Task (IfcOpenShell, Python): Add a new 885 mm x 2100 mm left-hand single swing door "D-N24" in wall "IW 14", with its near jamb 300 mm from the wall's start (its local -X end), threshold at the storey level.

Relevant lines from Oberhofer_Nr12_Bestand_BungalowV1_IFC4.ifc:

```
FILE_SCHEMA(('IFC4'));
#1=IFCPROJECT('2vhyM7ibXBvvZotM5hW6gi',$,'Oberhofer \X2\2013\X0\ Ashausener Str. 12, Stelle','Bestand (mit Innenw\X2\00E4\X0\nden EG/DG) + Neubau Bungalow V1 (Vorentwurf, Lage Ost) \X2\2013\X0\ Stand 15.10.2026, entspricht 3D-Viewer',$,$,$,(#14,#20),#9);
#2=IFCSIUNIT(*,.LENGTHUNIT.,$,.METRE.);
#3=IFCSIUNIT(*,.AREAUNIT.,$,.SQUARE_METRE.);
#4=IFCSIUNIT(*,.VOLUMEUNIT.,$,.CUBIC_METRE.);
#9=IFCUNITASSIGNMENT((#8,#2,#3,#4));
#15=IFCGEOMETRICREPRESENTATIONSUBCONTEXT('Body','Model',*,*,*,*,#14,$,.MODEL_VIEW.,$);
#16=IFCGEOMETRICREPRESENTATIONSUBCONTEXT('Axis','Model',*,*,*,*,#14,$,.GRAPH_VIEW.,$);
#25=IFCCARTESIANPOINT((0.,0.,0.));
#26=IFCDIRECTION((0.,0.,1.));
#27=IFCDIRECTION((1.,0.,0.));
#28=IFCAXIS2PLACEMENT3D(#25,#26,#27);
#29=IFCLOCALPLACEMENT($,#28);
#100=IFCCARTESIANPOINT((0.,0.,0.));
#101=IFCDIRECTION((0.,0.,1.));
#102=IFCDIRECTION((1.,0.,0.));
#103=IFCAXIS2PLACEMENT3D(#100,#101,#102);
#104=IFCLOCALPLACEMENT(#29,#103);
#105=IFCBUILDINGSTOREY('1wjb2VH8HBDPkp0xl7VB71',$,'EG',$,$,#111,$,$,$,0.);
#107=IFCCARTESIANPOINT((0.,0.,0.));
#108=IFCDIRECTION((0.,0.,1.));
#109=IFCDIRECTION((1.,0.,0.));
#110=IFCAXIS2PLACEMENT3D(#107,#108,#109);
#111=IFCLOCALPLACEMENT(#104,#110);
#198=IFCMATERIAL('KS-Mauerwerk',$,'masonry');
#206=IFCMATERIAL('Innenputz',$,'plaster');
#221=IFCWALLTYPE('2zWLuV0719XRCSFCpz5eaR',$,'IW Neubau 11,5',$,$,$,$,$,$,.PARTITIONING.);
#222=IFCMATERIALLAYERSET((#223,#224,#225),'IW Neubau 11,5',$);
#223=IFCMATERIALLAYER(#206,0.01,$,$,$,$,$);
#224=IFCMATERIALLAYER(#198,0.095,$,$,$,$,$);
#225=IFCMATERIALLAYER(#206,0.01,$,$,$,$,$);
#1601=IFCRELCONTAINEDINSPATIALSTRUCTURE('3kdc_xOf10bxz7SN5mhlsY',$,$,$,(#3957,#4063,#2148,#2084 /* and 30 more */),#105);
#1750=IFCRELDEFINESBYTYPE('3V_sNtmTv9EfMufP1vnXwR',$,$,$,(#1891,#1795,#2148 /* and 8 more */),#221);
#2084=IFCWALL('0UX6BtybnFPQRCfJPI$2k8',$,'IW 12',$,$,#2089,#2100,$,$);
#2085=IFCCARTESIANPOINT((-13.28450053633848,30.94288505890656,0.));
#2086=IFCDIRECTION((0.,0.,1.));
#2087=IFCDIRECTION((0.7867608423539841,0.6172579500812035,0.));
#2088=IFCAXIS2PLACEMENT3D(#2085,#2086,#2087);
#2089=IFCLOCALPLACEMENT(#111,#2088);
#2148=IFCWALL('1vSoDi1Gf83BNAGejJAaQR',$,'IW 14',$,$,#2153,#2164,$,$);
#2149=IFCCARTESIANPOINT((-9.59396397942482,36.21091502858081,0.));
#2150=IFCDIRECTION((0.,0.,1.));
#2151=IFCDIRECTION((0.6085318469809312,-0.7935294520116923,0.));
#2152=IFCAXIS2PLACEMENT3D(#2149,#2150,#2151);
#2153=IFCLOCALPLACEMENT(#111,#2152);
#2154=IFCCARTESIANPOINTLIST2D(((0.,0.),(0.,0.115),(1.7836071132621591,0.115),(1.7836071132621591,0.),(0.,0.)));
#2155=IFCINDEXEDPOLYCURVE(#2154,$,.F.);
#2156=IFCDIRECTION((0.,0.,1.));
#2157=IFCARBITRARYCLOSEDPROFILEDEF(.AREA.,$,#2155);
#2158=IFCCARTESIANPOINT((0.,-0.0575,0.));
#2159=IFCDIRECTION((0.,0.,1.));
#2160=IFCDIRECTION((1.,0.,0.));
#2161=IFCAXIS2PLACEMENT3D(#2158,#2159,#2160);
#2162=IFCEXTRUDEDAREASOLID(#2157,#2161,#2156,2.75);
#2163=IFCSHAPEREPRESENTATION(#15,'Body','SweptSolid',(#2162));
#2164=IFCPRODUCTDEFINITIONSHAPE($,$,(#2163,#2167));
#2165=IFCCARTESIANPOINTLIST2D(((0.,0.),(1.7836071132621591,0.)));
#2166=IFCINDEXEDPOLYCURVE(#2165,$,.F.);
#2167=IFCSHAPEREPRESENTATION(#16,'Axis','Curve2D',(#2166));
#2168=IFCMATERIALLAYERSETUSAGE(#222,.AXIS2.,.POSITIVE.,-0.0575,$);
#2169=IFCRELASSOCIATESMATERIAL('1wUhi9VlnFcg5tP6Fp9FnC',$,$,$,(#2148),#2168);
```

```python
import numpy as np
import ifcopenshell
import ifcopenshell.api.feature
import ifcopenshell.api.geometry
import ifcopenshell.api.root
import ifcopenshell.api.spatial
import ifcopenshell.geom
import ifcopenshell.util.element
import ifcopenshell.util.placement
import ifcopenshell.util.representation
import ifcopenshell.util.shape
import ifcopenshell.util.unit

model = ifcopenshell.open("Oberhofer_Nr12_Bestand_BungalowV1_IFC4.ifc")
unit_scale = ifcopenshell.util.unit.calculate_unit_scale(model)
settings = ifcopenshell.geom.settings()


def volume(element):
    """Net volume in cubic metres, openings subtracted."""
    shape = ifcopenshell.geom.create_shape(settings, element)
    return ifcopenshell.util.shape.get_volume(shape.geometry)


wall = model.by_guid("1vSoDi1Gf83BNAGejJAaQR")
storey = ifcopenshell.util.element.get_container(wall, ifc_class="IfcBuildingStorey")
context = ifcopenshell.util.representation.get_context(model, "Model", "Body", "MODEL_VIEW")
before = volume(wall)

width, height, from_end, sill = 0.885, 2.1, 0.3, 0.0  # metres

# The wall runs along its own X axis, and the end named is its -X end.
wall_shape = ifcopenshell.geom.create_shape(settings, wall)
x, y, z = ifcopenshell.util.shape.get_vertices(wall_shape.geometry).T
start = x.min() + from_end
face, thickness = float(y.min()), float(y.max() - y.min())
wall_matrix = ifcopenshell.util.placement.get_local_placement(wall.ObjectPlacement)
level = ifcopenshell.util.placement.get_local_placement(storey.ObjectPlacement)[2, 3]


def in_wall(x, y):
    """Placement at x, y metres in the wall's axes, at sill height."""
    matrix = wall_matrix.copy()
    matrix[:, 3] = wall_matrix @ np.array([x / unit_scale, y / unit_scale, 0.0, 1.0])
    matrix[2, 3] = level + sill / unit_scale
    return matrix


# Opening: a box that overshoots both wall faces by 50 mm.
opening = ifcopenshell.api.root.create_entity(model, ifc_class="IfcOpeningElement", predefined_type="OPENING")
box = ifcopenshell.api.geometry.add_wall_representation(
    model, context=context, length=width, height=height, thickness=thickness + 0.1
)
ifcopenshell.api.geometry.assign_representation(model, product=opening, representation=box)
ifcopenshell.api.geometry.edit_object_placement(model, product=opening, matrix=in_wall(start, face - 0.05), is_si=False)
ifcopenshell.api.feature.add_feature(model, feature=opening, element=wall)

door = ifcopenshell.api.root.create_entity(model, ifc_class="IfcDoor", name="D-N24", predefined_type="DOOR")
door.OverallWidth, door.OverallHeight = width / unit_scale, height / unit_scale
door.OperationType = "SINGLE_SWING_LEFT"
body = ifcopenshell.api.geometry.add_door_representation(
    model,
    context=context,
    overall_width=door.OverallWidth,
    overall_height=door.OverallHeight,
    operation_type="SINGLE_SWING_LEFT",
    lining_properties={"LiningDepth": thickness / unit_scale, "ThresholdDepth": thickness / unit_scale},
)
ifcopenshell.api.geometry.assign_representation(model, product=door, representation=body)
ifcopenshell.api.spatial.assign_container(model, products=[door], relating_structure=storey)
ifcopenshell.api.feature.add_filling(model, opening=opening, element=door)

# The lining spans the wall, so the door starts at the wall face.
ifcopenshell.api.geometry.edit_object_placement(model, product=door, matrix=in_wall(start, face), is_si=False)

after = volume(wall)

print(f"wall volume {before:.3f} -> {after:.3f} m3")

model.write("Oberhofer_Nr12_Bestand_BungalowV1_IFC4_rev.ifc")
```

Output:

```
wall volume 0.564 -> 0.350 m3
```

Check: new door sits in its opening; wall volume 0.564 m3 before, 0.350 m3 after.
